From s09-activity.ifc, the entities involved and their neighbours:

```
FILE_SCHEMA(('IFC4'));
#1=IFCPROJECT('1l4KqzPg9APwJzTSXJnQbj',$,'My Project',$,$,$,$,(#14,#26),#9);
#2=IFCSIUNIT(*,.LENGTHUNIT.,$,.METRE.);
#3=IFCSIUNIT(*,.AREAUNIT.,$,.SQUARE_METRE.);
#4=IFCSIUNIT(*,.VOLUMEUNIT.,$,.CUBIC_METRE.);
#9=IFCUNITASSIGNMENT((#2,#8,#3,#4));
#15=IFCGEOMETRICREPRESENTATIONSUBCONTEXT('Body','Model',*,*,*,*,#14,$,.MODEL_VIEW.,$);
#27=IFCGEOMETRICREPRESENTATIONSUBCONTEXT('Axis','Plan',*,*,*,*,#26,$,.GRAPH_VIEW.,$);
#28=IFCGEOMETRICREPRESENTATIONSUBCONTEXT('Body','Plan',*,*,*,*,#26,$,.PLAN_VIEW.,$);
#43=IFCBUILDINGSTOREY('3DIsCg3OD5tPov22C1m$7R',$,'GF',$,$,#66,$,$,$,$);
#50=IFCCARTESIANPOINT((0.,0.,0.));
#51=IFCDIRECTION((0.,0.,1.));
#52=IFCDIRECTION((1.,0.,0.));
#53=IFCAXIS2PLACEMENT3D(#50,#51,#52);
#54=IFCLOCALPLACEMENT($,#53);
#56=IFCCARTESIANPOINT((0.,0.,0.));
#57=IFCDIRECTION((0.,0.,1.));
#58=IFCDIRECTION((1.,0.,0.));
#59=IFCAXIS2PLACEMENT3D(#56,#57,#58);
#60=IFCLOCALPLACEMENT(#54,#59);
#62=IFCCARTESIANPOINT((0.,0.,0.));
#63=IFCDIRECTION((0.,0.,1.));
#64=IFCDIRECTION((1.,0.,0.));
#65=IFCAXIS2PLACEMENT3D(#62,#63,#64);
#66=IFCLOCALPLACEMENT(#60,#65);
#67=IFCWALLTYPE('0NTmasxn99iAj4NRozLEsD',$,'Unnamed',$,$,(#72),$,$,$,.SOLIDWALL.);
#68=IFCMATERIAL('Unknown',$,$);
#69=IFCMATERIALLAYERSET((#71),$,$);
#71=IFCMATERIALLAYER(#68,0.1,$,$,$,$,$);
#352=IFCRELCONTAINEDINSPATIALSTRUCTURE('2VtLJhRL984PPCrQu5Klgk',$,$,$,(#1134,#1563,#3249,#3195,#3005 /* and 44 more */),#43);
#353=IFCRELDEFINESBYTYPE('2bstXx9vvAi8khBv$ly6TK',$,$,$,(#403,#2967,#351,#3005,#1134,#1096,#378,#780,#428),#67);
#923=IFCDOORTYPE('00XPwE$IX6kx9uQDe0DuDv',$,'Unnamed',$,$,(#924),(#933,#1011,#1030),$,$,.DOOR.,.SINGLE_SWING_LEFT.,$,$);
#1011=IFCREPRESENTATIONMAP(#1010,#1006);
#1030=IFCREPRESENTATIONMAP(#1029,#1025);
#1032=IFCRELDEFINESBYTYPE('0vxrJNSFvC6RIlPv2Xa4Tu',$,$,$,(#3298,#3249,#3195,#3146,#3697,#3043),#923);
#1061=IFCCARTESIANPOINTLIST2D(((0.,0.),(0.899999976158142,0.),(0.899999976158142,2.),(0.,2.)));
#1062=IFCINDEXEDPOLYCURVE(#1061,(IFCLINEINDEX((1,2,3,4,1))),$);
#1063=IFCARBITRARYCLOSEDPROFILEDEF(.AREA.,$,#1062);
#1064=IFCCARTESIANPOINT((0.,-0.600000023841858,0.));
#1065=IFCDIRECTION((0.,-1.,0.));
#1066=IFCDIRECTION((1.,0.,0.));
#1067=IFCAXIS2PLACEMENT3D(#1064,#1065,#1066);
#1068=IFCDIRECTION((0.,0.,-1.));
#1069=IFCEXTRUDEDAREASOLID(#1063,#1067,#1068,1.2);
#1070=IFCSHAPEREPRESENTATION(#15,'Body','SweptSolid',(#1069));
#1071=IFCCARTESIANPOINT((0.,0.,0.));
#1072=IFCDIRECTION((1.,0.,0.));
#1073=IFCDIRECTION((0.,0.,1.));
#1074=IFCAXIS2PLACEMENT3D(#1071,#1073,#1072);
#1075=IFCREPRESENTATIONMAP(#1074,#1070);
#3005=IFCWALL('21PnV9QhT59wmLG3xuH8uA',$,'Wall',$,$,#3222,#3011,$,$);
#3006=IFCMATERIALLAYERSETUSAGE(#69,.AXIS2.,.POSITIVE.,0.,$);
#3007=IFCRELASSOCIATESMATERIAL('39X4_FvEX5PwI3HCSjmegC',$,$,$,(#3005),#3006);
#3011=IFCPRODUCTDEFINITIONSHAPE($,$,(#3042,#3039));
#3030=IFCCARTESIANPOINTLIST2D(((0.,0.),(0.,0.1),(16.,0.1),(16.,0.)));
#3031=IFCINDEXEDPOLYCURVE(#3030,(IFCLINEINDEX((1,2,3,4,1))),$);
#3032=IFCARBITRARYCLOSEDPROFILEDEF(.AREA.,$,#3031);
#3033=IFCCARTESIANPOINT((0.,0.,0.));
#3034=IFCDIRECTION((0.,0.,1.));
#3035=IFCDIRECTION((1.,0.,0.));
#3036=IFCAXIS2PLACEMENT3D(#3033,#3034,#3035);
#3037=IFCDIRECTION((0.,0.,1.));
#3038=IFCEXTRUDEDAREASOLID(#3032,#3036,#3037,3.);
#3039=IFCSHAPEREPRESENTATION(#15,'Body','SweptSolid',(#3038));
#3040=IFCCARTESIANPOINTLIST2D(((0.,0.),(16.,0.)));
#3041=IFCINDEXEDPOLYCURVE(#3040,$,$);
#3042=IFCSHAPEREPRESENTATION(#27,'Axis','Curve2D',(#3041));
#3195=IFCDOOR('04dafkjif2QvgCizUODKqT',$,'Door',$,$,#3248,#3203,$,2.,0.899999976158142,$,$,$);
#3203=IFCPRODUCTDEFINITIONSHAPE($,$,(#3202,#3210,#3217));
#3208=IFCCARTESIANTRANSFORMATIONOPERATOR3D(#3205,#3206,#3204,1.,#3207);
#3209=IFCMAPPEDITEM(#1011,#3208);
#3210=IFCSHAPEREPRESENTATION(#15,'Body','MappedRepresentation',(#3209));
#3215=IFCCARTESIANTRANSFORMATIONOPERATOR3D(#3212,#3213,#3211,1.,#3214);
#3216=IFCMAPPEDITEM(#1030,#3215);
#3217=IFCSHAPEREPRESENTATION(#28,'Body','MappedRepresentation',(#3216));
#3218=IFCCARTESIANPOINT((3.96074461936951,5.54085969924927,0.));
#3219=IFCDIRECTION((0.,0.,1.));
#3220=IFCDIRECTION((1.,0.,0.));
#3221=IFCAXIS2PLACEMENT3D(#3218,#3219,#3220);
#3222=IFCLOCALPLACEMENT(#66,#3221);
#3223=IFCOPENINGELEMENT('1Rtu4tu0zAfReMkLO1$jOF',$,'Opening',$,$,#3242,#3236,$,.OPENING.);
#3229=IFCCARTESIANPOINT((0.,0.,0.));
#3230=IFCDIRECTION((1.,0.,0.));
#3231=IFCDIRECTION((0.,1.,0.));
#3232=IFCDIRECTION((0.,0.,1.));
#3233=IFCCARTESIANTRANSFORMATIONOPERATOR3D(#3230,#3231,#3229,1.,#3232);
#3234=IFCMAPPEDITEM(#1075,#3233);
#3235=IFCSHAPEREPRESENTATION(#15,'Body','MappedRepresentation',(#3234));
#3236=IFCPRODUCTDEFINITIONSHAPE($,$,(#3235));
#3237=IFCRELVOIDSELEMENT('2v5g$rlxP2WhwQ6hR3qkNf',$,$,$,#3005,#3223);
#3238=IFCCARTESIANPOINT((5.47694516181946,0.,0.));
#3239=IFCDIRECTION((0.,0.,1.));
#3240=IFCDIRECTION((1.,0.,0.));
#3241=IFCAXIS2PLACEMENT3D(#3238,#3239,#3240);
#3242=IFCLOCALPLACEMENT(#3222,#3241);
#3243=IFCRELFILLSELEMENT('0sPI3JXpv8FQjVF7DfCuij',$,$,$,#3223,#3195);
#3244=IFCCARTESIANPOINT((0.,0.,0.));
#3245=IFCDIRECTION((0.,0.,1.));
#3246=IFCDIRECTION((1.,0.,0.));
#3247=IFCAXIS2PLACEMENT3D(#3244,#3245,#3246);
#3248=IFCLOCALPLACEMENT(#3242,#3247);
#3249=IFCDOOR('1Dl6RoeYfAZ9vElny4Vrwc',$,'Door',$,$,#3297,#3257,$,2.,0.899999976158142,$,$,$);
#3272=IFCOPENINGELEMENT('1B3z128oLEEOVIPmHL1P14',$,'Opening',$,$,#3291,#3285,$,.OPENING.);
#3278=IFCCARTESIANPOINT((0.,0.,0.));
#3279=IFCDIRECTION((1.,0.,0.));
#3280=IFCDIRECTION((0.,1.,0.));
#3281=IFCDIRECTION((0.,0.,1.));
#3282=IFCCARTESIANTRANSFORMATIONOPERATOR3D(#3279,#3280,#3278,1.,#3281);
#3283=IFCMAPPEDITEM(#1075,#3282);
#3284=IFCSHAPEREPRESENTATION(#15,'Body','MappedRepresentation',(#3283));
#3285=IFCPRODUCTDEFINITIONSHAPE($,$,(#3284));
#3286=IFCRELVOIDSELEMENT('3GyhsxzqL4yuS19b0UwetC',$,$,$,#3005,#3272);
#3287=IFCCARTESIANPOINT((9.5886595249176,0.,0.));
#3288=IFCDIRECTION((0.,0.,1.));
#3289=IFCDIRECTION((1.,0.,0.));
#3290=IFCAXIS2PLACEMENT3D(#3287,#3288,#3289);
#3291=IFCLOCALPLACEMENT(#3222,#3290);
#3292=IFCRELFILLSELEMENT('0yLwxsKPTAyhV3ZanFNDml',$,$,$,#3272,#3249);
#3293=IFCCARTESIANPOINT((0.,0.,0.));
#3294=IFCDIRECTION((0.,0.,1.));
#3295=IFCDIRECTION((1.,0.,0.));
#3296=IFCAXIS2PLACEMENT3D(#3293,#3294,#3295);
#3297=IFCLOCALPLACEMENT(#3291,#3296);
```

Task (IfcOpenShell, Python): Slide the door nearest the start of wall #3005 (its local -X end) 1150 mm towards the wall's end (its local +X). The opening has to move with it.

```python
import ifcopenshell
import ifcopenshell.api.geometry
import ifcopenshell.util.placement

model = ifcopenshell.open("s09-activity.ifc")

door = model.by_guid("04dafkjif2QvgCizUODKqT")
opening = door.FillsVoids[0].RelatingOpeningElement
wall = opening.VoidsElements[0].RelatingBuildingElement

wall_matrix = ifcopenshell.util.placement.get_local_placement(wall.ObjectPlacement)
shift = wall_matrix[:3, 0] * 1.15
before = ifcopenshell.util.placement.get_local_placement(door.ObjectPlacement)[:3, 3].copy()

# The door is placed relative to its opening, so it follows when the opening moves.
matrix = ifcopenshell.util.placement.get_local_placement(opening.ObjectPlacement)
matrix[:3, 3] += shift
ifcopenshell.api.geometry.edit_object_placement(
    model, product=opening, matrix=matrix, is_si=False, should_transform_children=True
)

after = ifcopenshell.util.placement.get_local_placement(door.ObjectPlacement)[:3, 3]
print("door moved by", (after - before).round(3) + 0.0)

model.write("s09-activity_edited.ifc")
```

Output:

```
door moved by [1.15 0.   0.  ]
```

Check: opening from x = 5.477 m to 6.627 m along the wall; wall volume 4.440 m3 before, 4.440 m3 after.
